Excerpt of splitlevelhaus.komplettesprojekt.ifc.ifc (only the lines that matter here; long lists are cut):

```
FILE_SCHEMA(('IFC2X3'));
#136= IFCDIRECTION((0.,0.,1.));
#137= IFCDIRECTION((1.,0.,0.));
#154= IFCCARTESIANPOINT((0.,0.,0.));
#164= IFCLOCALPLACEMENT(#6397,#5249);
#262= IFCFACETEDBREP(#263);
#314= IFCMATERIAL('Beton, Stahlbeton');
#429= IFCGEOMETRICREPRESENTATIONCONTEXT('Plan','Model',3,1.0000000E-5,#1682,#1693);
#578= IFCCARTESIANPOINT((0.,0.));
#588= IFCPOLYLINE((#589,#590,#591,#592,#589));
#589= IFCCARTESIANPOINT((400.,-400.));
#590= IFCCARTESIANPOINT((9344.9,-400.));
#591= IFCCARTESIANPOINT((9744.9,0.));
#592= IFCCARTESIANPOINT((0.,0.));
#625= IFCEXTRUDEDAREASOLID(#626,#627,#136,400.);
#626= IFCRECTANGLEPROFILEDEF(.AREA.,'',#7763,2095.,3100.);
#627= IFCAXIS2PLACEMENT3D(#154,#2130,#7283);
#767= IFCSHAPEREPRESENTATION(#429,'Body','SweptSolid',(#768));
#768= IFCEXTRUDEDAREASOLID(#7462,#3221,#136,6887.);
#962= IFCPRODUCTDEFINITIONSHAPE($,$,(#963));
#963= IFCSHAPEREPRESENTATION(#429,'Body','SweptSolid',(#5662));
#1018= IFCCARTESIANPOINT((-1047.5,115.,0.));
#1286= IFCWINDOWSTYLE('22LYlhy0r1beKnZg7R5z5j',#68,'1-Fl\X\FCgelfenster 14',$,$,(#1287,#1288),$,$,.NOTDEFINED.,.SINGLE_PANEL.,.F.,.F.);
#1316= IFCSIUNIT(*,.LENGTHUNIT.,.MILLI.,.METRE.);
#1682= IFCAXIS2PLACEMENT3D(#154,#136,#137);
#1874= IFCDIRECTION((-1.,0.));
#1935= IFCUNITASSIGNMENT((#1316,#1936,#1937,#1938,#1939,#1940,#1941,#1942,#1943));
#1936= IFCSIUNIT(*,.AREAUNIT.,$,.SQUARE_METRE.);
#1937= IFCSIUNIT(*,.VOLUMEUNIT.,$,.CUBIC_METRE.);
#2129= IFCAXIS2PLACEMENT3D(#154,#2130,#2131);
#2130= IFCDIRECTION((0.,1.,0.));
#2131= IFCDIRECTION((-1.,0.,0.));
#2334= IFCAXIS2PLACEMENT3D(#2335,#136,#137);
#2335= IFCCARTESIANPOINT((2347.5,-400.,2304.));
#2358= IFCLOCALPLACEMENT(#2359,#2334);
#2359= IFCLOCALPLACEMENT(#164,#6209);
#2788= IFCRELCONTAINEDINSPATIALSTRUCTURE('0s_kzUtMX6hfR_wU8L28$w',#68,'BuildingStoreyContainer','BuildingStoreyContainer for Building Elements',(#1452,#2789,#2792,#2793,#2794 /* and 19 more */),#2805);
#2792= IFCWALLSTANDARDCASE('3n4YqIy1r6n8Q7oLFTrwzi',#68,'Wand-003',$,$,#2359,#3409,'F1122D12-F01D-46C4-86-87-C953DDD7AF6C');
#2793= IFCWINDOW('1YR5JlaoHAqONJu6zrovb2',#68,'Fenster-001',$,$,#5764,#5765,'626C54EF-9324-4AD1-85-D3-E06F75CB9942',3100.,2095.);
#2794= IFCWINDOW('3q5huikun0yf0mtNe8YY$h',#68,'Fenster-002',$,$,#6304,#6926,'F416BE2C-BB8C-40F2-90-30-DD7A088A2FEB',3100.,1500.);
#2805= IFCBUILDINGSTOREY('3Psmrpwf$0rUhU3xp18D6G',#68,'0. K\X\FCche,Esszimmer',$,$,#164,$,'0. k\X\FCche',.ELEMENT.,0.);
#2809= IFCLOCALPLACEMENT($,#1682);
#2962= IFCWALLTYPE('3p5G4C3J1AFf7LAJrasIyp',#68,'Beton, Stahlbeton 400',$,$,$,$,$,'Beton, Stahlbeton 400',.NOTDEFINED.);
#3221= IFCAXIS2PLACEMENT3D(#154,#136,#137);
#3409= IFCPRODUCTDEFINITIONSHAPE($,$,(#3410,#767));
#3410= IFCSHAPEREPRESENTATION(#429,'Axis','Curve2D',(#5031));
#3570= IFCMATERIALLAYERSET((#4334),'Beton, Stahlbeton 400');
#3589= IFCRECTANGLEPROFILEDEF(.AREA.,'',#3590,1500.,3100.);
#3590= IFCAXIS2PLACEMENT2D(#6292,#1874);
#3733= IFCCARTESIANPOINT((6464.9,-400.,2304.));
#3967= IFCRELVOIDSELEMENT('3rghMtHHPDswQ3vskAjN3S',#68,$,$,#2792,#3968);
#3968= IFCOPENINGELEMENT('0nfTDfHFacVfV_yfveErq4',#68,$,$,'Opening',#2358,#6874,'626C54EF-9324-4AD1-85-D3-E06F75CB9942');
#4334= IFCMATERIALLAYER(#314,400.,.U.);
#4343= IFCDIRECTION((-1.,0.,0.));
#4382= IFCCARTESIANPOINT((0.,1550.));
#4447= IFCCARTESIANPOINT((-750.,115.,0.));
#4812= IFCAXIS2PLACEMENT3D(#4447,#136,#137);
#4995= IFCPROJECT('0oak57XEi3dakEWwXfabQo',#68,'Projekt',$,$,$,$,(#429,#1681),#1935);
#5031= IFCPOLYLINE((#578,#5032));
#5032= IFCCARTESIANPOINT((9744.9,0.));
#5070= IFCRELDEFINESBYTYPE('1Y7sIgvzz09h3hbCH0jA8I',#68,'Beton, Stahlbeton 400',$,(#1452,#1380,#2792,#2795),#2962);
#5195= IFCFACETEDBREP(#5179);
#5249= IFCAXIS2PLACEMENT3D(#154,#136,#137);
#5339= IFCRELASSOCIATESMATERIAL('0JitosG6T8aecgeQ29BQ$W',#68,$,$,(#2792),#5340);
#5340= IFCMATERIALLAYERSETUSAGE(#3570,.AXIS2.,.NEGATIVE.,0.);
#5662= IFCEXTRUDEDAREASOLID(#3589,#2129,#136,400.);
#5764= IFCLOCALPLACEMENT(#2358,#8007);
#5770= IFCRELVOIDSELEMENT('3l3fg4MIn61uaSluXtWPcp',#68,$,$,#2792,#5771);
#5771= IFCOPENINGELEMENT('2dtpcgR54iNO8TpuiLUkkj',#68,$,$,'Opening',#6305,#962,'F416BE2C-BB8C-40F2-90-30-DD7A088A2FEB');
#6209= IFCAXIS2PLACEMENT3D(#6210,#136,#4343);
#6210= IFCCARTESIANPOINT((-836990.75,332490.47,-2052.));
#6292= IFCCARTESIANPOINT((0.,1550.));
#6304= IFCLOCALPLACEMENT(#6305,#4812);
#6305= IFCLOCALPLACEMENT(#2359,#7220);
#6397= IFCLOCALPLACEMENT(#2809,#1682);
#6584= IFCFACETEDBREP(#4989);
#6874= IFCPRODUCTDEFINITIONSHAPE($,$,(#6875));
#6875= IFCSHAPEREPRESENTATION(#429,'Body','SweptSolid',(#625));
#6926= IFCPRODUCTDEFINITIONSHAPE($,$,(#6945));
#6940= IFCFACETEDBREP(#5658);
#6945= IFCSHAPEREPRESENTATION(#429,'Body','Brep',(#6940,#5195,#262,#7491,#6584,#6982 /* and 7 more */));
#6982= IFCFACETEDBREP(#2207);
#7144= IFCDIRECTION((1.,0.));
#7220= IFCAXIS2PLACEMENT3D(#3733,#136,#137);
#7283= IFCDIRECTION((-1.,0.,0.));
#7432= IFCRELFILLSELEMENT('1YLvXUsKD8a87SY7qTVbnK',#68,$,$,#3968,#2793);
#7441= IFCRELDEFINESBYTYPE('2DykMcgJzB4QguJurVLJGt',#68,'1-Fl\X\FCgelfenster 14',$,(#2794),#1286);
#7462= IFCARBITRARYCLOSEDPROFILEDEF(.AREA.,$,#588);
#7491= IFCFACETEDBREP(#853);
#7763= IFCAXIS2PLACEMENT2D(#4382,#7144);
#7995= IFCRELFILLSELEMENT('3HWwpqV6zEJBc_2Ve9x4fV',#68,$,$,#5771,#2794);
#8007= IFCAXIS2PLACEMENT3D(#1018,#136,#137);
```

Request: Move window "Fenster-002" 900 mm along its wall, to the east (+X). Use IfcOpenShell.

```python
import ifcopenshell
import ifcopenshell.api.geometry
import ifcopenshell.util.placement
import ifcopenshell.util.unit

model = ifcopenshell.open("splitlevelhaus.komplettesprojekt.ifc.ifc")
unit_scale = ifcopenshell.util.unit.calculate_unit_scale(model)

window = model.by_guid("3q5huikun0yf0mtNe8YY$h")
opening = window.FillsVoids[0].RelatingOpeningElement
wall = opening.VoidsElements[0].RelatingBuildingElement

wall_matrix = ifcopenshell.util.placement.get_local_placement(wall.ObjectPlacement)
shift = wall_matrix[:3, 0] * -0.9 / unit_scale
before = ifcopenshell.util.placement.get_local_placement(window.ObjectPlacement)[:3, 3].copy()

# The window is placed relative to its opening, so it follows when the opening moves.
matrix = ifcopenshell.util.placement.get_local_placement(opening.ObjectPlacement)
matrix[:3, 3] += shift
ifcopenshell.api.geometry.edit_object_placement(
    model, product=opening, matrix=matrix, is_si=False, should_transform_children=True
)

after = ifcopenshell.util.placement.get_local_placement(window.ObjectPlacement)[:3, 3]
print("window moved by", (after - before).round(3) + 0.0)

model.write("splitlevelhaus.komplettesprojekt.ifc_rev.ifc")
```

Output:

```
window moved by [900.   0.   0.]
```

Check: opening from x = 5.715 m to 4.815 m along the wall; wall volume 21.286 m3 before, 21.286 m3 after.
